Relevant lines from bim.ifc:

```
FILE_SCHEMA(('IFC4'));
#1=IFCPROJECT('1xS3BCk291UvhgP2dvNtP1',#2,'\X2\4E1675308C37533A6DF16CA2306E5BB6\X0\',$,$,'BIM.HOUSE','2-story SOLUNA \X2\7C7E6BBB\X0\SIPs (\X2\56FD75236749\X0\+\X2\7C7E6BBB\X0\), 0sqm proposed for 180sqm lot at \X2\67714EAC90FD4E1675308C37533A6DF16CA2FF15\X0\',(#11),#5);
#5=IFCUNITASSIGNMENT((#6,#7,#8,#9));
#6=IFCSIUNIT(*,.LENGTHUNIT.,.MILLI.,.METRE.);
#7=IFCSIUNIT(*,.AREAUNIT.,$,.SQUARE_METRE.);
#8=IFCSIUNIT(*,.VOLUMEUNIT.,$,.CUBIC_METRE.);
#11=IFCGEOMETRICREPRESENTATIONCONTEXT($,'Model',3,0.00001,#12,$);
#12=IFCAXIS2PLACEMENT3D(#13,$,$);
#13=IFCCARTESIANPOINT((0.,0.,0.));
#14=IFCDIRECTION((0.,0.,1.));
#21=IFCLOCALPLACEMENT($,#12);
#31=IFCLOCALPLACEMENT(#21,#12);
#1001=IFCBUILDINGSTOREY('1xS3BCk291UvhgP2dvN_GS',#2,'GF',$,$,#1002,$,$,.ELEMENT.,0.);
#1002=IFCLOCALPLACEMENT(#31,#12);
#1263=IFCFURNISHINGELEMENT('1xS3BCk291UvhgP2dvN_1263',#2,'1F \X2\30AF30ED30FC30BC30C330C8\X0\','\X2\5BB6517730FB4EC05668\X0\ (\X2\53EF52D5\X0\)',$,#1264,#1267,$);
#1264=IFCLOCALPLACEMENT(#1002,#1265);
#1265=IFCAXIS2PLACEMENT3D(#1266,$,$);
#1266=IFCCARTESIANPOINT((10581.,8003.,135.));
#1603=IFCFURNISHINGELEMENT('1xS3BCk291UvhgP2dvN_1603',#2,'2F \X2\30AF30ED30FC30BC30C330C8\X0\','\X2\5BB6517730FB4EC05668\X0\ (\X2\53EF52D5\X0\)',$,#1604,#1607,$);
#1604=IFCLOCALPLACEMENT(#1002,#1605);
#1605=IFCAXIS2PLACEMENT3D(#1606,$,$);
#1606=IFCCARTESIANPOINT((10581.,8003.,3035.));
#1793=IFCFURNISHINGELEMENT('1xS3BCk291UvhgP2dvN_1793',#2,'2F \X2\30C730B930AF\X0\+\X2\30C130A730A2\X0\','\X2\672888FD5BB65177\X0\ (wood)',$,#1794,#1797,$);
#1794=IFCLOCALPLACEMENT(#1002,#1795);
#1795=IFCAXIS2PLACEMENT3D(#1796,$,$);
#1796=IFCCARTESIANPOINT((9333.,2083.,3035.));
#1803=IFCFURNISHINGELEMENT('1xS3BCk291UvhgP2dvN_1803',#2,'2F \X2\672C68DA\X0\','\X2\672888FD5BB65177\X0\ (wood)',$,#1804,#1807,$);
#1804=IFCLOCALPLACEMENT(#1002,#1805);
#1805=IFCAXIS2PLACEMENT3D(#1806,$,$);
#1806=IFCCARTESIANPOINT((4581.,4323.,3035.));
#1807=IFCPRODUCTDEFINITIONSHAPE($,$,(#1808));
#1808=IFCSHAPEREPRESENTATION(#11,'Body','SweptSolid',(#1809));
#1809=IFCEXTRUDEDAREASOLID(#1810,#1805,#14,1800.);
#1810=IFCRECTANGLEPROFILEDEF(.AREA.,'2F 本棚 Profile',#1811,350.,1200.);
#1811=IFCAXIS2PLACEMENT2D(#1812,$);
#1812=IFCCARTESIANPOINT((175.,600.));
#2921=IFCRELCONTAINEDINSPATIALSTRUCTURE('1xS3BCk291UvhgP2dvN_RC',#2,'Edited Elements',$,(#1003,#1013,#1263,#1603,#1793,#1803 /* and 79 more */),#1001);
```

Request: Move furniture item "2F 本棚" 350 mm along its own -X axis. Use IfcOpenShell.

```python
import ifcopenshell
import ifcopenshell.api.geometry
import ifcopenshell.util.placement
import ifcopenshell.util.unit

model = ifcopenshell.open("bim.ifc")
unit_scale = ifcopenshell.util.unit.calculate_unit_scale(model)

item = model.by_guid("1xS3BCk291UvhgP2dvN_1803")
matrix = ifcopenshell.util.placement.get_local_placement(item.ObjectPlacement)
matrix[:3, 3] -= matrix[:3, 0] * 0.35 / unit_scale
ifcopenshell.api.geometry.edit_object_placement(model, product=item, matrix=matrix, is_si=False)

print(ifcopenshell.util.placement.get_local_placement(item.ObjectPlacement).round(3) + 0.0)

model.write("bim_v2.ifc")
```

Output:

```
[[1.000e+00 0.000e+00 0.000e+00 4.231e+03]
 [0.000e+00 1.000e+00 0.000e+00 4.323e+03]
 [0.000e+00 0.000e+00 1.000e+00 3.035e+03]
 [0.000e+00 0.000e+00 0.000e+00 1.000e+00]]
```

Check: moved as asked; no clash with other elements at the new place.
